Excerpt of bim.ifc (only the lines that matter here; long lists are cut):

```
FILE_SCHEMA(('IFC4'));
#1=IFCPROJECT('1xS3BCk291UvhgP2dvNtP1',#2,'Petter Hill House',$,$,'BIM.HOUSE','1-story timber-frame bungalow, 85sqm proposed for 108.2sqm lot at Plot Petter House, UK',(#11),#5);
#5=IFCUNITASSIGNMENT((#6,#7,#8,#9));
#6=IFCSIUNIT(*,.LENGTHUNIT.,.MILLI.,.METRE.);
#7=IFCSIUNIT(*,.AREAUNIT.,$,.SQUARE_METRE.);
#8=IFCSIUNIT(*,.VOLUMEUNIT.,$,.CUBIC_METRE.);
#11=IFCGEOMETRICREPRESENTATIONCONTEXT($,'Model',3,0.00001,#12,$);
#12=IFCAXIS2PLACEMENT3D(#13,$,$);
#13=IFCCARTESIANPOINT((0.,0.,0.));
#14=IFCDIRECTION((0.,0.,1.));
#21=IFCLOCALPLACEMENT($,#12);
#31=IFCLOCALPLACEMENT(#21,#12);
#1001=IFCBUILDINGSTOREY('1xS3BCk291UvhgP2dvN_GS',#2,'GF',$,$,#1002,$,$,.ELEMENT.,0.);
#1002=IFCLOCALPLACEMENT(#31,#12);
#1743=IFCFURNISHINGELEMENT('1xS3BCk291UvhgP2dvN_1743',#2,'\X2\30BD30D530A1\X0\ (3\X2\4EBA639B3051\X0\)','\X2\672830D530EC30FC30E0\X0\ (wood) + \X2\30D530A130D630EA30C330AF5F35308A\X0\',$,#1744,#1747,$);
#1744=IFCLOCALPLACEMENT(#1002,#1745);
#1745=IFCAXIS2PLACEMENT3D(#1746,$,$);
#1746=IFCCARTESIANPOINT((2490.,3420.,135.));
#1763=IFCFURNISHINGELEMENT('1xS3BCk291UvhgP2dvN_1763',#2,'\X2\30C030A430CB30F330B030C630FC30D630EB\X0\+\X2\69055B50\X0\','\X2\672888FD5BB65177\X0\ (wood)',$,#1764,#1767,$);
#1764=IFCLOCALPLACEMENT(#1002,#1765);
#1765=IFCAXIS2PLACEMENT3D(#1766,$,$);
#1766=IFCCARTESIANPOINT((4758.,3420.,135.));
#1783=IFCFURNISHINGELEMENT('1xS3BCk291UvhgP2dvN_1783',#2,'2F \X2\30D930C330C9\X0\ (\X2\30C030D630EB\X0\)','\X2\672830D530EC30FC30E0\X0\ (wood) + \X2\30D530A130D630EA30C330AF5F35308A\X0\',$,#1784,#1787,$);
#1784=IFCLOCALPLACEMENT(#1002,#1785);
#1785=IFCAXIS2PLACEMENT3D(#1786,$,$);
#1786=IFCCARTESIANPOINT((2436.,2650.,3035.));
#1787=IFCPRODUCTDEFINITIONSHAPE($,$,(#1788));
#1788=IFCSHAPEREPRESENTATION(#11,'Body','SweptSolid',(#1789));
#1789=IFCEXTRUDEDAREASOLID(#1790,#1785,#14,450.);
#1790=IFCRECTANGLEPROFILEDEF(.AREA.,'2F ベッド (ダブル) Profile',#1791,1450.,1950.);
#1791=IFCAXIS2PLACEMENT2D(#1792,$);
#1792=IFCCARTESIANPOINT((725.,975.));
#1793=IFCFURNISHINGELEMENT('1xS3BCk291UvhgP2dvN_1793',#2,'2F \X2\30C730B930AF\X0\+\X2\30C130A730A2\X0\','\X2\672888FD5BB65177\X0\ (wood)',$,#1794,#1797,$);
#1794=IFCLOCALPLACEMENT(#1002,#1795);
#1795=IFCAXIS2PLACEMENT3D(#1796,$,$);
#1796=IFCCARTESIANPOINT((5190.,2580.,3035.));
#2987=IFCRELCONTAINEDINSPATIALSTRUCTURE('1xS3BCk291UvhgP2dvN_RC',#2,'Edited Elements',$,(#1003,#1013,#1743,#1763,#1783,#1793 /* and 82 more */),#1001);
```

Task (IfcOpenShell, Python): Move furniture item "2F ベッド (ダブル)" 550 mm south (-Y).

```python
import ifcopenshell
import ifcopenshell.api.geometry
import ifcopenshell.util.placement

model = ifcopenshell.open("bim.ifc")

item = model.by_guid("1xS3BCk291UvhgP2dvN_1783")
matrix = ifcopenshell.util.placement.get_local_placement(item.ObjectPlacement)
matrix[1, 3] -= 550.0
ifcopenshell.api.geometry.edit_object_placement(model, product=item, matrix=matrix, is_si=False)

print(ifcopenshell.util.placement.get_local_placement(item.ObjectPlacement).round(3) + 0.0)

model.write("bim-out.ifc")
```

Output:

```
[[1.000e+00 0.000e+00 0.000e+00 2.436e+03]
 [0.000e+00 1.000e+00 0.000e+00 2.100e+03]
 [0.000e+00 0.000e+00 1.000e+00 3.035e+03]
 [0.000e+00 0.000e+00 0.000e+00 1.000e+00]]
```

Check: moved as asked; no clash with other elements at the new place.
